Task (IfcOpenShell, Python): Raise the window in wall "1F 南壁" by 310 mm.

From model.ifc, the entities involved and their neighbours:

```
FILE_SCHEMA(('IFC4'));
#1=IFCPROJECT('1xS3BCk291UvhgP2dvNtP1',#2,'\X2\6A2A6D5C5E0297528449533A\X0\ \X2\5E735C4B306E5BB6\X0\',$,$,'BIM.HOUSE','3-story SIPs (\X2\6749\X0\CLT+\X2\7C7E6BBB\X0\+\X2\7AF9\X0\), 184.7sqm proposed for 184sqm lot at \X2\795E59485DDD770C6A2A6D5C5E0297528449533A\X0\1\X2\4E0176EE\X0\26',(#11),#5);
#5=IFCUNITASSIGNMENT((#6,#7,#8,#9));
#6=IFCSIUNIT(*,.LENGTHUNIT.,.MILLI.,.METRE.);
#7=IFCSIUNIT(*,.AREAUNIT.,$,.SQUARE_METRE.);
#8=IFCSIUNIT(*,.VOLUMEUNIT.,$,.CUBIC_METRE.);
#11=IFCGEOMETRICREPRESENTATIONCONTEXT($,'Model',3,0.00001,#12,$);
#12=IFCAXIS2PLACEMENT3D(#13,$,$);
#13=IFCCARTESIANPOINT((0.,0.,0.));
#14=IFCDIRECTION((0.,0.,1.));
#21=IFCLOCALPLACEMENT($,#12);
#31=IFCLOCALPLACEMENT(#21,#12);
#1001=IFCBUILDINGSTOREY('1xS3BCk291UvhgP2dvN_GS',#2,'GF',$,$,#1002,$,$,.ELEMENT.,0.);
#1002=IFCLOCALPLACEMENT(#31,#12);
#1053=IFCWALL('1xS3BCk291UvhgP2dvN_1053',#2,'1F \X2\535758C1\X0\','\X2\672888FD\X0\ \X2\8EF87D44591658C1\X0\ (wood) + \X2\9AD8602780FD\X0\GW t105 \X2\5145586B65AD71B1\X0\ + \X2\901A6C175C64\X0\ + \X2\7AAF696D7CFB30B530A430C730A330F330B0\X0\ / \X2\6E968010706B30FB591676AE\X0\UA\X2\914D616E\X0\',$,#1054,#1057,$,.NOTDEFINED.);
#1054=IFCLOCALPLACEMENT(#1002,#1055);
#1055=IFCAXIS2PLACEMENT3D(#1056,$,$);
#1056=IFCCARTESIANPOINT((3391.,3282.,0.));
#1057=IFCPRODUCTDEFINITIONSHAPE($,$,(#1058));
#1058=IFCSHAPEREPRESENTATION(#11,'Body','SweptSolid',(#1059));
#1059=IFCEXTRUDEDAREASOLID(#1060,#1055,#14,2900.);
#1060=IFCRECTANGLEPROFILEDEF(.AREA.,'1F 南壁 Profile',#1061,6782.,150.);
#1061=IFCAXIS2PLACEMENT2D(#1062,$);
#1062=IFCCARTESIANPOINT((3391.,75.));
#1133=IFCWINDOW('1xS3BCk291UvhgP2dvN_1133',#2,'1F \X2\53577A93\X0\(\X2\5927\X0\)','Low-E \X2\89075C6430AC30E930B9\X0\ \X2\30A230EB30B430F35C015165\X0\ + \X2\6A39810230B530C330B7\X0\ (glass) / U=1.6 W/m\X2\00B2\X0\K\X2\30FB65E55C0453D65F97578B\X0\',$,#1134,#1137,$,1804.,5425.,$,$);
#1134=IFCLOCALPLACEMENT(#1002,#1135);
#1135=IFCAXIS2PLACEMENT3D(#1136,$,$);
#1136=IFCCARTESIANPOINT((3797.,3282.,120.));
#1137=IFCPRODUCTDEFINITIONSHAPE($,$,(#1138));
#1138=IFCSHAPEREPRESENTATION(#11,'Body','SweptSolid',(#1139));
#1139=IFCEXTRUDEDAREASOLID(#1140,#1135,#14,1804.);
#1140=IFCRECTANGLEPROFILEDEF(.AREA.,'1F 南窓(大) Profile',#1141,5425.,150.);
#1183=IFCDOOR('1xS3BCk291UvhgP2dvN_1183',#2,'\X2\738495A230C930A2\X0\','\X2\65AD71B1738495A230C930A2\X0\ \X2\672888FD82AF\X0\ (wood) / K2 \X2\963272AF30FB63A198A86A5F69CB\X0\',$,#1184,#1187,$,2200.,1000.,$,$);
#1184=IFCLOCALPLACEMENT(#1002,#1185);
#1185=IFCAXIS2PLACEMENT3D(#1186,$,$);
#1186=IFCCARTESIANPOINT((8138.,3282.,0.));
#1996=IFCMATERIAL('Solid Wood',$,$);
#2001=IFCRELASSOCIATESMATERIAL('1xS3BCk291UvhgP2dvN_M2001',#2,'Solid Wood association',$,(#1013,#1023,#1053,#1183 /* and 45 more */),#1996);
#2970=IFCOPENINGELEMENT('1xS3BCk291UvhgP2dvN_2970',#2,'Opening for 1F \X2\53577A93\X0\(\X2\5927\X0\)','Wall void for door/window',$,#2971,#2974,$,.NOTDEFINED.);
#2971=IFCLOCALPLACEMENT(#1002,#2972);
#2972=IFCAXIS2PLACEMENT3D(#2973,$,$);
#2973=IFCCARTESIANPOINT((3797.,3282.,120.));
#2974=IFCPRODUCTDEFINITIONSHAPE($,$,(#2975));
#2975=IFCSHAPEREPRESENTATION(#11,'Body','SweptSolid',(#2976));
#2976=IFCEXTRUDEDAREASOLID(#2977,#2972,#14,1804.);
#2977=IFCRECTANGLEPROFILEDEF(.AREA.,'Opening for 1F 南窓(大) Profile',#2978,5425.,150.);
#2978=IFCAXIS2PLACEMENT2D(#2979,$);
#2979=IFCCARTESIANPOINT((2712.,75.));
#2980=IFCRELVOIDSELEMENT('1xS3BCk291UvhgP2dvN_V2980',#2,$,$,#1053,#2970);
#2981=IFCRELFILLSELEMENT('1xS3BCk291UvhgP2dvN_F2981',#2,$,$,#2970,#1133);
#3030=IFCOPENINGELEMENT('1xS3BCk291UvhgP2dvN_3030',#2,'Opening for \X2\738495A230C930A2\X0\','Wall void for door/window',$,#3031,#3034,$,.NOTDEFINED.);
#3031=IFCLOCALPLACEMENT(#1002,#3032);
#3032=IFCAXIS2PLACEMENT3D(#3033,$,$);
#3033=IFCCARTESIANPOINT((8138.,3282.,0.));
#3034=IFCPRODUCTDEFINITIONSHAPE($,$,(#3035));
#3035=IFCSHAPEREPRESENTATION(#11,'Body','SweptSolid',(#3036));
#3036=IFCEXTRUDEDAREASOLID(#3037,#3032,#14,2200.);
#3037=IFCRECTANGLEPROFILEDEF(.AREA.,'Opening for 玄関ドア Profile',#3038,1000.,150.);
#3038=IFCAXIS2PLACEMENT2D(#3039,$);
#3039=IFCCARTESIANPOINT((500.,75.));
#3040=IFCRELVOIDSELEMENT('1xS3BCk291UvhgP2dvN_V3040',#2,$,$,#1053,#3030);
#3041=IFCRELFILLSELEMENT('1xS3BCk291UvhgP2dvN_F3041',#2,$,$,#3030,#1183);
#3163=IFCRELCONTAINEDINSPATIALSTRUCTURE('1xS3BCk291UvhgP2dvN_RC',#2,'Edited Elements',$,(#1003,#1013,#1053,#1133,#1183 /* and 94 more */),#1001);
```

```python
import numpy as np
import ifcopenshell
import ifcopenshell.api.geometry
import ifcopenshell.util.placement
import ifcopenshell.util.unit

model = ifcopenshell.open("model.ifc")
unit_scale = ifcopenshell.util.unit.calculate_unit_scale(model)

window = model.by_guid("1xS3BCk291UvhgP2dvN_1133")
opening = window.FillsVoids[0].RelatingOpeningElement
dz = 310.0

shift = np.array([0.0, 0.0, dz])
# The window is not placed relative to its opening, so move both.
for product in (opening, window):
    matrix = ifcopenshell.util.placement.get_local_placement(product.ObjectPlacement)
    matrix[:3, 3] += shift
    ifcopenshell.api.geometry.edit_object_placement(model, product=product, matrix=matrix, is_si=False)

print(f"moved by {dz * unit_scale:+.3f} m")

model.write("model_v2.ifc")
```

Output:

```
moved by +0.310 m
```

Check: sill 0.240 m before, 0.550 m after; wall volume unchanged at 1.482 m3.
